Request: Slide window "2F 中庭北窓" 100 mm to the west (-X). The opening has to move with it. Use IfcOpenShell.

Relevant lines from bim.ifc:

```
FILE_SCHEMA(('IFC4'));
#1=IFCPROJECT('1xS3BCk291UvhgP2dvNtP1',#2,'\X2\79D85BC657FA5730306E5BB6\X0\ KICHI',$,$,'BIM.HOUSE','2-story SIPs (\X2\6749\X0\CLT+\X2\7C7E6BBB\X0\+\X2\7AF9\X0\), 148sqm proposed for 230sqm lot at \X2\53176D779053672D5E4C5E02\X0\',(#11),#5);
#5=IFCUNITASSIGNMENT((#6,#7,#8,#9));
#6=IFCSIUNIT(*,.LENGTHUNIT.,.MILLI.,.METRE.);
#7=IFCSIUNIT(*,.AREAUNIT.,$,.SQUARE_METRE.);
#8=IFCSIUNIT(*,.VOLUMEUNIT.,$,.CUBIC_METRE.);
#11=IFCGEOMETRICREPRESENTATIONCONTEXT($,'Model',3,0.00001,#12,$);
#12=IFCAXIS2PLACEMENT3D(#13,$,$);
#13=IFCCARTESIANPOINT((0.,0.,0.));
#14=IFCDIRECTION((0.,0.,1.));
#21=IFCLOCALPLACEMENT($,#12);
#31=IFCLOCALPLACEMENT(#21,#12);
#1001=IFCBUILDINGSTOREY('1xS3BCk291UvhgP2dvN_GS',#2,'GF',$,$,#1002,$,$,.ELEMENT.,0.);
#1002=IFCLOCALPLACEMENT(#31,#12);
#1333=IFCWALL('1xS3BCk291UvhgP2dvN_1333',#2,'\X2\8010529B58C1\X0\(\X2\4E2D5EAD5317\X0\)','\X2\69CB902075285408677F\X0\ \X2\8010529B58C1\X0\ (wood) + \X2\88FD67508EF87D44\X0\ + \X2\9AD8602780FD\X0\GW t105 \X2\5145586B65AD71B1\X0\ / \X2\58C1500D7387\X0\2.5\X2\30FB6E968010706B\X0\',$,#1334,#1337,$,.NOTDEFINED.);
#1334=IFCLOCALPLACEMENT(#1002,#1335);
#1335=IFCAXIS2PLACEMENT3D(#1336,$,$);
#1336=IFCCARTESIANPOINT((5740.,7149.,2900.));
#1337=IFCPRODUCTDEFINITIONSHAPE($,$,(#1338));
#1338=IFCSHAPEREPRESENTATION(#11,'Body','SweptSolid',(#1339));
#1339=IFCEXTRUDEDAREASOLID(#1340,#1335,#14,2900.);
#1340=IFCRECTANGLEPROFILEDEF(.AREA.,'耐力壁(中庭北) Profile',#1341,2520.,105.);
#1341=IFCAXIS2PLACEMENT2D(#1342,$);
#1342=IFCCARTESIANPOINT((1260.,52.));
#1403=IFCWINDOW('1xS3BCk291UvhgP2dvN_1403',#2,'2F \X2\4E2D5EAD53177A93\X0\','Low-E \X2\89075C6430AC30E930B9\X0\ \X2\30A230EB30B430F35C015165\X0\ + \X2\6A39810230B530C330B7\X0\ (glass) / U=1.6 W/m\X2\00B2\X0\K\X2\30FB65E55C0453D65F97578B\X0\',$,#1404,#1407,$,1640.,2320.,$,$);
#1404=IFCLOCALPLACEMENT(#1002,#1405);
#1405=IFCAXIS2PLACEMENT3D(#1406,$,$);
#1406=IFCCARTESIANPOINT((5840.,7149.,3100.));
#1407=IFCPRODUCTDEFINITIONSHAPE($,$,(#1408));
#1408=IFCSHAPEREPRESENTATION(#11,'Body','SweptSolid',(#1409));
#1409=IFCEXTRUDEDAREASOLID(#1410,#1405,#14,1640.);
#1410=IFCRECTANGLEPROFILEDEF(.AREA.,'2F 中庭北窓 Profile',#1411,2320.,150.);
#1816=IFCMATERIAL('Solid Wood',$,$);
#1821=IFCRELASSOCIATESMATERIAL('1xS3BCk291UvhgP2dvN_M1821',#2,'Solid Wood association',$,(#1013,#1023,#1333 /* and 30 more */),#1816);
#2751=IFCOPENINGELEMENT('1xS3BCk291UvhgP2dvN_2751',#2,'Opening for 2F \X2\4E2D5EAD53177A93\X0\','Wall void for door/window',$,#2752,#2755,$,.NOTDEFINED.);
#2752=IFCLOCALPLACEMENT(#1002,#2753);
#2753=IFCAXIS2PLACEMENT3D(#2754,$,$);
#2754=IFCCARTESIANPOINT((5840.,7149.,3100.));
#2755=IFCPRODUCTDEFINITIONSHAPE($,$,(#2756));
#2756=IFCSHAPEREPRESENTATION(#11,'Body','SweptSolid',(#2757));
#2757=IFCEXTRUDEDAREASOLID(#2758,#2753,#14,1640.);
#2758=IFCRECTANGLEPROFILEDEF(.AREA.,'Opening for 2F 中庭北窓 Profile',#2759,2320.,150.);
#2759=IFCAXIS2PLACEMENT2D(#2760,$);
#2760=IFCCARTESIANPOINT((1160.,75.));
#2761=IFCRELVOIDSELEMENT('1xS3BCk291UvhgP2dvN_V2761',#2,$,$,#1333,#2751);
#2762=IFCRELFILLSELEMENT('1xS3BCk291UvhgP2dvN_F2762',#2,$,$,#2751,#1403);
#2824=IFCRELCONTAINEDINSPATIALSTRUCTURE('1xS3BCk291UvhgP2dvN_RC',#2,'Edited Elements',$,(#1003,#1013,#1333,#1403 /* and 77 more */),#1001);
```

```python
import ifcopenshell
import ifcopenshell.api.geometry
import ifcopenshell.util.placement
import ifcopenshell.util.unit

model = ifcopenshell.open("bim.ifc")
unit_scale = ifcopenshell.util.unit.calculate_unit_scale(model)

window = model.by_id(1403)
opening = window.FillsVoids[0].RelatingOpeningElement
wall = opening.VoidsElements[0].RelatingBuildingElement

wall_matrix = ifcopenshell.util.placement.get_local_placement(wall.ObjectPlacement)
shift = wall_matrix[:3, 0] * -0.1 / unit_scale
before = ifcopenshell.util.placement.get_local_placement(window.ObjectPlacement)[:3, 3].copy()

# The window is not placed relative to its opening, so move both.
for product in (opening, window):
    matrix = ifcopenshell.util.placement.get_local_placement(product.ObjectPlacement)
    matrix[:3, 3] += shift
    ifcopenshell.api.geometry.edit_object_placement(model, product=product, matrix=matrix, is_si=False)

after = ifcopenshell.util.placement.get_local_placement(window.ObjectPlacement)[:3, 3]
print("window moved by", (after - before).round(3) + 0.0)

model.write("bim-out.ifc")
```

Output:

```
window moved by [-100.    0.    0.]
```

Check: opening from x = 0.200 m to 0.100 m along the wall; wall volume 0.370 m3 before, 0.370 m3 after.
